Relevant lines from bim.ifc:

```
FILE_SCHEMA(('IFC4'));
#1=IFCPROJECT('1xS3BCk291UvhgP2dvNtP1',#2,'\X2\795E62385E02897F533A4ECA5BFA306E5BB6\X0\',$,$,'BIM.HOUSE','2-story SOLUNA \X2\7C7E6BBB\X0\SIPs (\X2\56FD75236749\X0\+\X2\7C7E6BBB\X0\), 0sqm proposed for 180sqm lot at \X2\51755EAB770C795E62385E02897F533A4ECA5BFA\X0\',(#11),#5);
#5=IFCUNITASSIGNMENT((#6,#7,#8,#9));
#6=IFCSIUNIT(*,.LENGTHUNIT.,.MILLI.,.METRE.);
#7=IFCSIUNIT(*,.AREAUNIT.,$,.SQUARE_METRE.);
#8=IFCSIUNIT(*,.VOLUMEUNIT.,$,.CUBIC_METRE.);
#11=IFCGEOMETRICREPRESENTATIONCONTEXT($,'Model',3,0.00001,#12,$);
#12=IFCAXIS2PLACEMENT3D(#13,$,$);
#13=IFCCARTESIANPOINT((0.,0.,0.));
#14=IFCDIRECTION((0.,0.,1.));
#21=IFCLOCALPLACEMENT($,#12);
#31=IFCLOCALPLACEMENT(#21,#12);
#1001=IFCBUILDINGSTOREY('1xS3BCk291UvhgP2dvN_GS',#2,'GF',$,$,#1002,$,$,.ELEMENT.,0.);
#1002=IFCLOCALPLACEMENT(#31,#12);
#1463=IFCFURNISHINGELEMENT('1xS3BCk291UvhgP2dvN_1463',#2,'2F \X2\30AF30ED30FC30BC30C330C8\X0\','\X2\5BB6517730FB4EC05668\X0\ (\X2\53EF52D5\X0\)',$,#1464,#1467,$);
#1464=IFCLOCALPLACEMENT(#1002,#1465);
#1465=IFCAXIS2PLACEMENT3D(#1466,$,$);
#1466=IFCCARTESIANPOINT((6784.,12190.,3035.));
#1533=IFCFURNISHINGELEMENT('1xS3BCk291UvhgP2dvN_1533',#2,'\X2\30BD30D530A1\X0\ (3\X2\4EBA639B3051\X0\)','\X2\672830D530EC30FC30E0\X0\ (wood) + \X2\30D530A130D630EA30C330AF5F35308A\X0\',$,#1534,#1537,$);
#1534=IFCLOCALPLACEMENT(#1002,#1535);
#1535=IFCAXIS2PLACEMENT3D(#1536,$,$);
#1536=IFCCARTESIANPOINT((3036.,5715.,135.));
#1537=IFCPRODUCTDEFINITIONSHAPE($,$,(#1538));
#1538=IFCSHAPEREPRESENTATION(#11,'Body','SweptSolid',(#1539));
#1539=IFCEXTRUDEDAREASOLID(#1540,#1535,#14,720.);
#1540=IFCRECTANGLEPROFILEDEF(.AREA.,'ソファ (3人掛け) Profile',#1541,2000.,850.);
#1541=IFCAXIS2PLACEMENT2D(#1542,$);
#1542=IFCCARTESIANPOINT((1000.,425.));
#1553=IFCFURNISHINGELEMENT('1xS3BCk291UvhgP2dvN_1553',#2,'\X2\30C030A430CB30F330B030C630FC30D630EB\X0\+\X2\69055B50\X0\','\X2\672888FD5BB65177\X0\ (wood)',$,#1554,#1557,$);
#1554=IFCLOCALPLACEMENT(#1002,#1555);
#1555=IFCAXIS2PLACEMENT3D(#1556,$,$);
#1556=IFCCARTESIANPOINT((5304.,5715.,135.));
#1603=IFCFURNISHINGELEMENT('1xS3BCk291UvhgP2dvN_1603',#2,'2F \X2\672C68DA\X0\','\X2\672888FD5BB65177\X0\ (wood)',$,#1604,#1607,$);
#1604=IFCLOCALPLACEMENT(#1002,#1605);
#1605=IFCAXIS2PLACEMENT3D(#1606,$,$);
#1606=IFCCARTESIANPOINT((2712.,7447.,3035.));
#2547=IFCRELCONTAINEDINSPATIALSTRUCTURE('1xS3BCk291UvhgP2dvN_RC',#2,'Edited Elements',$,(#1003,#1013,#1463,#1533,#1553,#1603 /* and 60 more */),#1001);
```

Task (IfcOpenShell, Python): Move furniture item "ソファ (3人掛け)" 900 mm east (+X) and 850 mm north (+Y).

```python
import ifcopenshell
import ifcopenshell.api.geometry
import ifcopenshell.util.placement

model = ifcopenshell.open("bim.ifc")

item = model.by_guid("1xS3BCk291UvhgP2dvN_1533")
matrix = ifcopenshell.util.placement.get_local_placement(item.ObjectPlacement)
matrix[0, 3] += 900.0
matrix[1, 3] += 850.0
ifcopenshell.api.geometry.edit_object_placement(model, product=item, matrix=matrix, is_si=False)

print(ifcopenshell.util.placement.get_local_placement(item.ObjectPlacement).round(3) + 0.0)

model.write("bim_v2.ifc")
```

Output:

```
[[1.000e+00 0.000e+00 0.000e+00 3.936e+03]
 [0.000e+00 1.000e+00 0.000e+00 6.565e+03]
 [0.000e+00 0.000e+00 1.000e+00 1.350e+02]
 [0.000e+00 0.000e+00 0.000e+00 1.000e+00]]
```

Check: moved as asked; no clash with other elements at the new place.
